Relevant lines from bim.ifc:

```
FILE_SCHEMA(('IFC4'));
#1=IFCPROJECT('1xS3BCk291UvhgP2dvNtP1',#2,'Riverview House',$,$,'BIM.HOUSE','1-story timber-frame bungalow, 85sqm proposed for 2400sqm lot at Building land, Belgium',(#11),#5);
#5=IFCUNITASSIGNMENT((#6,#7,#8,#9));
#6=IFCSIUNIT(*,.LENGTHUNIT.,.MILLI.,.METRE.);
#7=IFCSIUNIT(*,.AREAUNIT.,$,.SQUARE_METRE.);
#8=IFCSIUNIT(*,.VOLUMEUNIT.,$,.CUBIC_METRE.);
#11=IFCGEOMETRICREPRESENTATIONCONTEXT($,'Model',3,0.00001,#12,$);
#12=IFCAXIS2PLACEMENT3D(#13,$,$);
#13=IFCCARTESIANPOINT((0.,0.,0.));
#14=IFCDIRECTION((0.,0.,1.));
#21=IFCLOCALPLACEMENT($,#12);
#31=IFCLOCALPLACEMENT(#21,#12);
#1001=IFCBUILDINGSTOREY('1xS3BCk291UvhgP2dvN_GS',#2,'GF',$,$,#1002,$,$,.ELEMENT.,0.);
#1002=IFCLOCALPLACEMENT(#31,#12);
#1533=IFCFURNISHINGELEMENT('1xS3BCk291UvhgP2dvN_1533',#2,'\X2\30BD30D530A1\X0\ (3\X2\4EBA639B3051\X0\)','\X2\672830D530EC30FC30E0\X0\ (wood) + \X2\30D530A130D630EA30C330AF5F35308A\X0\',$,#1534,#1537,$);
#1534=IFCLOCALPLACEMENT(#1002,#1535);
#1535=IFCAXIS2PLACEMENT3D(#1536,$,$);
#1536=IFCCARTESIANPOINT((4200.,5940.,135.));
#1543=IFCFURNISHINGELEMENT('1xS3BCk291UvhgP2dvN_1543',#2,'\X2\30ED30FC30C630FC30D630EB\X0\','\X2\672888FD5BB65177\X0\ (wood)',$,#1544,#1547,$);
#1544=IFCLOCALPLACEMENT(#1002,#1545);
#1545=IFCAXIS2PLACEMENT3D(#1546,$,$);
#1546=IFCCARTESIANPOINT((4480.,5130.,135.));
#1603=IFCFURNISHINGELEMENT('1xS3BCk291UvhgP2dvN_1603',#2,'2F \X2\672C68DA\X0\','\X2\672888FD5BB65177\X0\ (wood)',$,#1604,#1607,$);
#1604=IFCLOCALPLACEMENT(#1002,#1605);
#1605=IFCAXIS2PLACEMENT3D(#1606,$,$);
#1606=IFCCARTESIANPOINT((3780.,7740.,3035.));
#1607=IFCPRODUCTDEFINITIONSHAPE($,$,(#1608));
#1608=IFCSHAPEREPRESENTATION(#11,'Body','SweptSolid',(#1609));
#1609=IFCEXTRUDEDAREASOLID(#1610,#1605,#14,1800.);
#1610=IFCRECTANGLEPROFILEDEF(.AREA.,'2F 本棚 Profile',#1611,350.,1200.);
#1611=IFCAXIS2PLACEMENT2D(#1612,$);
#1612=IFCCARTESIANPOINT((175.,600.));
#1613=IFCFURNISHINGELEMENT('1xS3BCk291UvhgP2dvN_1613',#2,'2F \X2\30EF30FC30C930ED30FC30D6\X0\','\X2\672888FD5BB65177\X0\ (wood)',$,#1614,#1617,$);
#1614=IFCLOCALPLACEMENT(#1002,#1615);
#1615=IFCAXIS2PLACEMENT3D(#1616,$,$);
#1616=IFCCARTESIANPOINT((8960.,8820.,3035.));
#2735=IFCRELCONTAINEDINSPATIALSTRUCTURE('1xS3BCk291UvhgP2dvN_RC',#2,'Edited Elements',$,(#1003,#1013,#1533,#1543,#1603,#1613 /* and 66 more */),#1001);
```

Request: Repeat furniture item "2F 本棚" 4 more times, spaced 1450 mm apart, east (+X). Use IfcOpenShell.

```python
import numpy as np
import ifcopenshell
import ifcopenshell.api.geometry
import ifcopenshell.api.root
import ifcopenshell.util.element
import ifcopenshell.util.placement
import ifcopenshell.util.unit

model = ifcopenshell.open("bim.ifc")
unit_scale = ifcopenshell.util.unit.calculate_unit_scale(model)


def reuse_history(source, copy):
    """copy_class also copies each property set's owner history, people and application; keep the originals."""
    for rel in copy.IsDefinedBy:
        if rel.is_a("IfcRelDefinesByProperties") and (history := rel.RelatingPropertyDefinition.OwnerHistory):
            rel.RelatingPropertyDefinition.OwnerHistory = source.OwnerHistory
            ifcopenshell.util.element.remove_deep2(model, history)


source = model.by_id(1603)
base = ifcopenshell.util.placement.get_local_placement(source.ObjectPlacement)
step = np.array([1.0, 0.0, 0.0]) * 1.45 / unit_scale

for i in range(1, 5):
    copy = ifcopenshell.api.root.copy_class(model, product=source)
    copy.Representation = ifcopenshell.util.element.copy_deep(
        model, source.Representation, exclude=["IfcGeometricRepresentationContext", "IfcRepresentationMap"]
    )
    reuse_history(source, copy)
    matrix = base.copy()
    matrix[:3, 3] += i * step
    print("added at", matrix[:3, 3].round(3) + 0.0)
    ifcopenshell.api.geometry.edit_object_placement(model, product=copy, matrix=matrix, is_si=False)

model.write("bim_v2.ifc")
```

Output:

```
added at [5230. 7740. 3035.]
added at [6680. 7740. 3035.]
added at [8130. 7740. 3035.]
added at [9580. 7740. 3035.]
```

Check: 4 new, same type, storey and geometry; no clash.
